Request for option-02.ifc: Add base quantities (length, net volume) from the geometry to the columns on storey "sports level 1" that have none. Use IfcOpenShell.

First a look at what the model holds.

```python
import ifcopenshell
import ifcopenshell.util.element
import ifcopenshell.util.unit

model = ifcopenshell.open("option-02.ifc")
print(model.schema)
for unit_type in ("LENGTHUNIT", "AREAUNIT", "VOLUMEUNIT"):
    print(unit_type, ifcopenshell.util.unit.calculate_unit_scale(model, unit_type))
storey = next(s for s in model.by_type("IfcBuildingStorey") if s.Name == "sports level 1")
columns = [e for e in ifcopenshell.util.element.get_decomposition(storey) if e.is_a("IfcColumn")]
for e in sorted(columns, key=lambda e: e.id()):
    print(e.id(), e.is_a(), e.Name, list(ifcopenshell.util.element.get_psets(e, qtos_only=True)), sep=" | ")
```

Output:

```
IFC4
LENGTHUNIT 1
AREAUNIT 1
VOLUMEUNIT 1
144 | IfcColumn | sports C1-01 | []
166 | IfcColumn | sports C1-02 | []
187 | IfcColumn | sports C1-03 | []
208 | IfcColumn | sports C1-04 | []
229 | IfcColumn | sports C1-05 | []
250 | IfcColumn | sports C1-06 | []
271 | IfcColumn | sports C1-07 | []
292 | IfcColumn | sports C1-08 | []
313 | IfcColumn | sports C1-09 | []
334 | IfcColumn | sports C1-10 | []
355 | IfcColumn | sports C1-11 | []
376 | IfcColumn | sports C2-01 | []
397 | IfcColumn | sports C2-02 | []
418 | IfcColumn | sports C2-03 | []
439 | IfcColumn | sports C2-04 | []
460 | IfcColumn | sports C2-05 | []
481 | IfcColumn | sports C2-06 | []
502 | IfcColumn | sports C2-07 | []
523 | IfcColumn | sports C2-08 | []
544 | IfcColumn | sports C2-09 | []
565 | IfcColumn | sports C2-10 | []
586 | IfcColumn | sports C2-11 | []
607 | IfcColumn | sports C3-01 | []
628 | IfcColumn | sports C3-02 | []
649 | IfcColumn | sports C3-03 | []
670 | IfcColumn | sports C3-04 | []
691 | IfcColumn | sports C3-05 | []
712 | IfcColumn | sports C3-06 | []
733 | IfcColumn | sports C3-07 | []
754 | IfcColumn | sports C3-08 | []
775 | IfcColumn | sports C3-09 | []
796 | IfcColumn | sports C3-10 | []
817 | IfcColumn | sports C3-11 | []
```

```python
import ifcopenshell
import ifcopenshell.api.pset
import ifcopenshell.geom
import ifcopenshell.util.element
import ifcopenshell.util.shape
import ifcopenshell.util.unit

model = ifcopenshell.open("option-02.ifc")
unit_scale = ifcopenshell.util.unit.calculate_unit_scale(model)
volume_scale = ifcopenshell.util.unit.calculate_unit_scale(model, "VOLUMEUNIT")
settings = ifcopenshell.geom.settings()

storey = next(s for s in model.by_type("IfcBuildingStorey") if s.Name == "sports level 1")
columns = [e for e in ifcopenshell.util.element.get_decomposition(storey) if e.is_a("IfcColumn")]

for e in sorted(columns, key=lambda e: e.id()):
    if ifcopenshell.util.element.get_psets(e, qtos_only=True, should_inherit=False):
        continue
    # Geometry comes back in metres, in the element's own axes.
    shape = ifcopenshell.geom.create_shape(settings, e)
    values = {
        "Length": ifcopenshell.util.shape.get_z(shape.geometry) / unit_scale,
        "NetVolume": ifcopenshell.util.shape.get_volume(shape.geometry) / volume_scale,
    }
    qto = ifcopenshell.api.pset.add_qto(model, product=e, name="Qto_ColumnBaseQuantities")
    ifcopenshell.api.pset.edit_qto(model, qto=qto, properties=values)
    print(e.id(), {k: round(v, 3) for k, v in values.items()})

model.write("option-02_edited.ifc")
```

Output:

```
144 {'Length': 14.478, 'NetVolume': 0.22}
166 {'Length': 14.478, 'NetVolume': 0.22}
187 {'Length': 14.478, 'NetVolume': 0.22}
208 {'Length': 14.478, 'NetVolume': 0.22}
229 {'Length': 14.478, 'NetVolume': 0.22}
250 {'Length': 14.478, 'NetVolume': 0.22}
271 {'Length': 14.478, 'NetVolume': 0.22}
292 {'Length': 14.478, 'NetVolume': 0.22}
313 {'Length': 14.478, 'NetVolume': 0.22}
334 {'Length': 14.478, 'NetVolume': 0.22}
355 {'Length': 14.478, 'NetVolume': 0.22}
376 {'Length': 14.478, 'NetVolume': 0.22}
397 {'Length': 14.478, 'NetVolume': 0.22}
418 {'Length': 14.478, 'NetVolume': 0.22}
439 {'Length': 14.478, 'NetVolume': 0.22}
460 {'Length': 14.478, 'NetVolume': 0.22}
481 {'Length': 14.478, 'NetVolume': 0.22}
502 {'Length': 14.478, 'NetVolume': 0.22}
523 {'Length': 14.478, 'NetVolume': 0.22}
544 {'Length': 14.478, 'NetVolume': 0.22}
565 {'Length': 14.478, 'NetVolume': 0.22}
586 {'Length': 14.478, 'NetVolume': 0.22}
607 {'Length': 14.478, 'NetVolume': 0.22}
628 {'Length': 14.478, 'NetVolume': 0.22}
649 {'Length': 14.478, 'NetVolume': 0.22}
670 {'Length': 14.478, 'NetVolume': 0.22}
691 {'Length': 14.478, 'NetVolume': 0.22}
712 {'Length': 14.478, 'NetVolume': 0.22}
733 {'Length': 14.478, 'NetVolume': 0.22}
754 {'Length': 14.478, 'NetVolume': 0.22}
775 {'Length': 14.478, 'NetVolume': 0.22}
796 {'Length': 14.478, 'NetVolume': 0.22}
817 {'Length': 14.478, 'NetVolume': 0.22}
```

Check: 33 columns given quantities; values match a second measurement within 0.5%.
